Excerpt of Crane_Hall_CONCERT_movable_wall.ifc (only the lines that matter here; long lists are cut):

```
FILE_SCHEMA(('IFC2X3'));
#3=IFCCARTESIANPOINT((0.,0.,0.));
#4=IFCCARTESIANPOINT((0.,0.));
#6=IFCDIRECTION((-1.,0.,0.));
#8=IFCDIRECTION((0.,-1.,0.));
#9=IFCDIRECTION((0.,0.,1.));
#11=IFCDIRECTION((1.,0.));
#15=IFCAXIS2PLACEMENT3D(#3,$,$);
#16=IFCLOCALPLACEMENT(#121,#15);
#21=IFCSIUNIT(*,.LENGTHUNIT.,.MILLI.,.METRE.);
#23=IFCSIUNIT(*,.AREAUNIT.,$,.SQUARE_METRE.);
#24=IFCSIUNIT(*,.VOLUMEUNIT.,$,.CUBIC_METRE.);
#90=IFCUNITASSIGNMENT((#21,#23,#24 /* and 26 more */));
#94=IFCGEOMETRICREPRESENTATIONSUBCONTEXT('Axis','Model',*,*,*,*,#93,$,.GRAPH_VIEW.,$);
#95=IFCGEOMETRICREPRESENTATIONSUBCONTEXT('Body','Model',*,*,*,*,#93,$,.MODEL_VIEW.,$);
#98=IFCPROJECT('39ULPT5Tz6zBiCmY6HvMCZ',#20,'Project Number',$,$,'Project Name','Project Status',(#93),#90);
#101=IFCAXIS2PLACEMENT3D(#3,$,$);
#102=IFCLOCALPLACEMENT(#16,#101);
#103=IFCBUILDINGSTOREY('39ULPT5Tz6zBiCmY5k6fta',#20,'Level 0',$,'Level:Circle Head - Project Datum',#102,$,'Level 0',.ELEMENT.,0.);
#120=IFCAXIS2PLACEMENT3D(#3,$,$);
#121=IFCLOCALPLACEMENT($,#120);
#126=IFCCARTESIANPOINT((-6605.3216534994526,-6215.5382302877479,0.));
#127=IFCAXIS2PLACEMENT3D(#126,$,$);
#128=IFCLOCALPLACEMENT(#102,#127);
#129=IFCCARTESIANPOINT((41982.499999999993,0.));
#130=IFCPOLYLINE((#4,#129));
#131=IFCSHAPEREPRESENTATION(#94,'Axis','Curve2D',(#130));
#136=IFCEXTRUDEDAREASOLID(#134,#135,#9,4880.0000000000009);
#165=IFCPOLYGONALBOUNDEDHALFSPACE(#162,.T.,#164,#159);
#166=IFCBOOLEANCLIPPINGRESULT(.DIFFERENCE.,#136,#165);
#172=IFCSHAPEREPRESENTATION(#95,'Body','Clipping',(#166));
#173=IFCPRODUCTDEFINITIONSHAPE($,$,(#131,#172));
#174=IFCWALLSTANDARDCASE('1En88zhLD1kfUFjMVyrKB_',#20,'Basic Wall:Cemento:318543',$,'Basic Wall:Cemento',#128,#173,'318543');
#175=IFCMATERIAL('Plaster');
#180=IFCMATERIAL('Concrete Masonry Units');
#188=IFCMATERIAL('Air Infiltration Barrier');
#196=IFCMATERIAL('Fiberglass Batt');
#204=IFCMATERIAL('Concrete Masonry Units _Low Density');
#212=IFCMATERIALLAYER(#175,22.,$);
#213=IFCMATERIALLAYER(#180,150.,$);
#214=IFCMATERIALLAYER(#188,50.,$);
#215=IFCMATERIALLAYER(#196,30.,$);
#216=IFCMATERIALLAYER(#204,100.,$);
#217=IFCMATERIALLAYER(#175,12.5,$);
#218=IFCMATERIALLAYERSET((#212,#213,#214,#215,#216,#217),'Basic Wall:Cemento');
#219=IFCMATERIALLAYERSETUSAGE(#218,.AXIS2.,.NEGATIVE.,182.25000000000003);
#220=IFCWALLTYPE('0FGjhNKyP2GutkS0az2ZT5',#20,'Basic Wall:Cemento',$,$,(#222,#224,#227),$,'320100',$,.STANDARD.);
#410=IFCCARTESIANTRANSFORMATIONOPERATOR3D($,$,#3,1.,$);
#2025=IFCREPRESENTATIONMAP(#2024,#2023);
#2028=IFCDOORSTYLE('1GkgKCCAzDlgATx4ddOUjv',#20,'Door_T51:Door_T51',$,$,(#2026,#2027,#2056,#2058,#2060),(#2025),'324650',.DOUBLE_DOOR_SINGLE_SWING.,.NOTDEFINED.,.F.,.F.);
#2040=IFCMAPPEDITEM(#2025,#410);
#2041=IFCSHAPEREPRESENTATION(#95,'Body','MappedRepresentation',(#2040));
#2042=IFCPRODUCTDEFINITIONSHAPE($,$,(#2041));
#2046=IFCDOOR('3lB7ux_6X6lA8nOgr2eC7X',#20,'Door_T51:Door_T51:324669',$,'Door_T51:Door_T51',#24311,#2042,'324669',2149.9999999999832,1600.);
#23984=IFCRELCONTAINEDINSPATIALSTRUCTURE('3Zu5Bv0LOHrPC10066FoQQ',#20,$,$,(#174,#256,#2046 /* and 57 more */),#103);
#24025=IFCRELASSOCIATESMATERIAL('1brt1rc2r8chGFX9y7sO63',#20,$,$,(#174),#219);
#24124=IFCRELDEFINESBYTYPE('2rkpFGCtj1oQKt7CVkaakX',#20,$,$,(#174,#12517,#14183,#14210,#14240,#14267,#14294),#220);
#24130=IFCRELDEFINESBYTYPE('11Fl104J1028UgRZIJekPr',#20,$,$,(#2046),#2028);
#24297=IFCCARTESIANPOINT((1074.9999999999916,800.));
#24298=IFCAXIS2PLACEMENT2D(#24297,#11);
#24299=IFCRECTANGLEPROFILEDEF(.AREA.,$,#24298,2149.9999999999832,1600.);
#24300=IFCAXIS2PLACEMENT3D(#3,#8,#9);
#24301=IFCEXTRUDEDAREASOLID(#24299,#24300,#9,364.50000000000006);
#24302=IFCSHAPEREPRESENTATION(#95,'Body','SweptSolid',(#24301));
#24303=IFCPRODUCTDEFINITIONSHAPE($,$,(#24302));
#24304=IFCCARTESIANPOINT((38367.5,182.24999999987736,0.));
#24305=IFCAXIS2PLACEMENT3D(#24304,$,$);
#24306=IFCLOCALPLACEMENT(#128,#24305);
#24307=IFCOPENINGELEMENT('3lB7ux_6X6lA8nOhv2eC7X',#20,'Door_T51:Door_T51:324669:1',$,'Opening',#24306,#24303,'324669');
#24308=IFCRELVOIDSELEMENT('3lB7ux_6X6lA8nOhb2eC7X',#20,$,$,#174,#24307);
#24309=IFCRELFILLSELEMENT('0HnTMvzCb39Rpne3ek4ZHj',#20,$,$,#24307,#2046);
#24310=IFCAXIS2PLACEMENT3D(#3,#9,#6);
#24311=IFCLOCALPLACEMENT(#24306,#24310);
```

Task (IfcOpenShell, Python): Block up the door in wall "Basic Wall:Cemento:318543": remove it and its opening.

```python
import ifcopenshell
import ifcopenshell.api.feature
import ifcopenshell.api.root
import ifcopenshell.geom
import ifcopenshell.util.shape

model = ifcopenshell.open("Crane_Hall_CONCERT_movable_wall.ifc")
settings = ifcopenshell.geom.settings()


def volume(element):
    """Net volume in cubic metres, openings subtracted."""
    shape = ifcopenshell.geom.create_shape(settings, element)
    return ifcopenshell.util.shape.get_volume(shape.geometry)


door = model.by_guid("3lB7ux_6X6lA8nOgr2eC7X")
opening = door.FillsVoids[0].RelatingOpeningElement
wall = opening.VoidsElements[0].RelatingBuildingElement
before = volume(wall)

ifcopenshell.api.root.remove_product(model, product=door)
ifcopenshell.api.feature.remove_feature(model, feature=opening)

after = volume(wall)

print(f"wall volume {before:.3f} -> {after:.3f} m3")

model.write("Crane_Hall_CONCERT_movable_wall_v2.ifc")
```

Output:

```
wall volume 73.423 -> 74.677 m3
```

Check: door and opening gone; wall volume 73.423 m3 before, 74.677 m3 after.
